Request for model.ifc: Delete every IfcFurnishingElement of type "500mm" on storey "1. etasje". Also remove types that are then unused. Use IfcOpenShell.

First a look at what the model holds.

```python
import ifcopenshell
import ifcopenshell.util.element

model = ifcopenshell.open("model.ifc")
print(model.schema)
storey = next(s for s in model.by_type("IfcBuildingStorey") if s.Name == "1. etasje")
furniture = [e for e in ifcopenshell.util.element.get_decomposition(storey) if e.is_a("IfcFurnishingElement")]
seen = {}
for e in furniture:
    element_type = ifcopenshell.util.element.get_type(e)
    name = element_type.Name if element_type not in (None, e) else None
    seen[name] = seen.get(name, 0) + 1
for name, count in sorted(seen.items(), key=str):
    print(count, "x", name)
```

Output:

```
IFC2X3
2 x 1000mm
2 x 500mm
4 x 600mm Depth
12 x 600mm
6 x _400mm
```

```python
import ifcopenshell
import ifcopenshell.api.root
import ifcopenshell.util.element

model = ifcopenshell.open("model.ifc")

storey = next(s for s in model.by_type("IfcBuildingStorey") if s.Name == "1. etasje")
furniture = [e for e in ifcopenshell.util.element.get_decomposition(storey) if e.is_a("IfcFurnishingElement")]
targets = [e for e in furniture if (t := ifcopenshell.util.element.get_type(e)) not in (None, e) and t.Name == "500mm"]
types = {ifcopenshell.util.element.get_type(e) for e in targets} - {None, *targets}

for e in targets:
    ifcopenshell.api.root.remove_product(model, product=e)
print(len(targets), "removed")

unused = [t for t in types if not ifcopenshell.util.element.get_types(t)]
for t in unused:
    ifcopenshell.api.root.remove_product(model, product=t)
print(len(unused), "unused types removed")

model.write("model-out.ifc")
```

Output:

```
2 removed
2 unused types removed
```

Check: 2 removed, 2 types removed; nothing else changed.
